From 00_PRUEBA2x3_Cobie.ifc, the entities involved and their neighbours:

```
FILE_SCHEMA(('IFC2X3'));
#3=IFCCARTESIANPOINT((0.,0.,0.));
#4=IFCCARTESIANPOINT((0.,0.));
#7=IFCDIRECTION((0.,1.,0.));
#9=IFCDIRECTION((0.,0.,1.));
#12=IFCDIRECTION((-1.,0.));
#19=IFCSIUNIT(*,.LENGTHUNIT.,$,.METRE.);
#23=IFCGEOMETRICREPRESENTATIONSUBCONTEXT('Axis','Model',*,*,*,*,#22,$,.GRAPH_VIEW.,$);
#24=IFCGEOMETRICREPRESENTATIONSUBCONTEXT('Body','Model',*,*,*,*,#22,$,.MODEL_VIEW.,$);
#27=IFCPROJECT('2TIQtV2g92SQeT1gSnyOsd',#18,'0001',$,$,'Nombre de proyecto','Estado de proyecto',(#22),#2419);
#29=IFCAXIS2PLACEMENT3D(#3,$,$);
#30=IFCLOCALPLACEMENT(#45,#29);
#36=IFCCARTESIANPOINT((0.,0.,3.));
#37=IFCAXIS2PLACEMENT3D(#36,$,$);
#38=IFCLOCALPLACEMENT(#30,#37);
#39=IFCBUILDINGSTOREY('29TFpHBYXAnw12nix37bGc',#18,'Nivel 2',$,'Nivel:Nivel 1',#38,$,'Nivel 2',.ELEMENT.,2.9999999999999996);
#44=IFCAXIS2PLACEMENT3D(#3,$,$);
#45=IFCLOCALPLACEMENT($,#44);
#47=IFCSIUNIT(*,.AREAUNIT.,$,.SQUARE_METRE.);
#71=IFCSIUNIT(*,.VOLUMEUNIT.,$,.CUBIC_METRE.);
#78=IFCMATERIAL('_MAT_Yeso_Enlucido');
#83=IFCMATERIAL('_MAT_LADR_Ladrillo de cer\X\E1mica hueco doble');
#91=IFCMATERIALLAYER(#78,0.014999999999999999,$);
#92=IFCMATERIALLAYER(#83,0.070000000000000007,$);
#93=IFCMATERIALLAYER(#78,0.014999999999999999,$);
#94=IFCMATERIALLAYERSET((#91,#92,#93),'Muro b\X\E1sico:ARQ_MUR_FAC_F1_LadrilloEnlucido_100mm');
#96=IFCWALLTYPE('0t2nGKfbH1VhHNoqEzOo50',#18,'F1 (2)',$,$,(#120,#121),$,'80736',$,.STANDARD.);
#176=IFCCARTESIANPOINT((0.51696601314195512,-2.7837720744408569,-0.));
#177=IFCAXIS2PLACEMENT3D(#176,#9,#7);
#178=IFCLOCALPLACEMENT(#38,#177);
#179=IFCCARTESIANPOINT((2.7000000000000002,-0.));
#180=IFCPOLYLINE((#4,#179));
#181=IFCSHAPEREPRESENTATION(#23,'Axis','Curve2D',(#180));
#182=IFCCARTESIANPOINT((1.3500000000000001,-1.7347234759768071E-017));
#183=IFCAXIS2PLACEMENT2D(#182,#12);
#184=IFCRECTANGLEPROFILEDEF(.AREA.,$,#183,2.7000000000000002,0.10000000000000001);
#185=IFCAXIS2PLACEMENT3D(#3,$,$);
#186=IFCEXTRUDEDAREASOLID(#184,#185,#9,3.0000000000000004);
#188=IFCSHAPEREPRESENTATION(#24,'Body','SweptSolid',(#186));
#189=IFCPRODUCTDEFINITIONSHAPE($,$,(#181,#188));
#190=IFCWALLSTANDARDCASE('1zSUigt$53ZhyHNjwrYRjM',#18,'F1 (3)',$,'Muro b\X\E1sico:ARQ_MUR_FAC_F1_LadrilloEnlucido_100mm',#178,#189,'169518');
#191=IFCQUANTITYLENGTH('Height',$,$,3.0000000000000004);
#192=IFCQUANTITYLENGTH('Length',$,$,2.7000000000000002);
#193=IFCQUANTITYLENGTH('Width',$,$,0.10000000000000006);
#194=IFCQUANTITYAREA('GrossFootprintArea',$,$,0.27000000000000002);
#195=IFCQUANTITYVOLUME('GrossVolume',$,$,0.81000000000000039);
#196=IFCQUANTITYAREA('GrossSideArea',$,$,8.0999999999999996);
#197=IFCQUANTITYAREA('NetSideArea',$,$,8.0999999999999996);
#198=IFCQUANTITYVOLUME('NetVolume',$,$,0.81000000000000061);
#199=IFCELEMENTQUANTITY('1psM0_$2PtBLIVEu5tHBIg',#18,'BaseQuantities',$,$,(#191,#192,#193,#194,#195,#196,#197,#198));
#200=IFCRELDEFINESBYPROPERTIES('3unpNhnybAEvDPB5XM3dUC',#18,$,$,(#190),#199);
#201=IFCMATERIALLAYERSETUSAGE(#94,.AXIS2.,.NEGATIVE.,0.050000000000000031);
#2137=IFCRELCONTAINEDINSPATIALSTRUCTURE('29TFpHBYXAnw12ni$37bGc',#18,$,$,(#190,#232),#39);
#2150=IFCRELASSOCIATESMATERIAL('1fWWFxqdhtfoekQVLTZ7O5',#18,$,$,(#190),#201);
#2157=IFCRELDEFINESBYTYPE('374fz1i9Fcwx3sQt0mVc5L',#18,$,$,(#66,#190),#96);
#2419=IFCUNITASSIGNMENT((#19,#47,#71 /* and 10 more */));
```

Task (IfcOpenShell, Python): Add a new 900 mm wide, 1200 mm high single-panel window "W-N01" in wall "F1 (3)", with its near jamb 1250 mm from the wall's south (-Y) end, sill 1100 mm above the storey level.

```python
import numpy as np
import ifcopenshell
import ifcopenshell.api.feature
import ifcopenshell.api.geometry
import ifcopenshell.api.pset
import ifcopenshell.api.root
import ifcopenshell.api.spatial
import ifcopenshell.api.type
import ifcopenshell.geom
import ifcopenshell.util.element
import ifcopenshell.util.placement
import ifcopenshell.util.representation
import ifcopenshell.util.shape
import ifcopenshell.util.unit

model = ifcopenshell.open("00_PRUEBA2x3_Cobie.ifc")
unit_scale = ifcopenshell.util.unit.calculate_unit_scale(model)
area_scale = ifcopenshell.util.unit.calculate_unit_scale(model, "AREAUNIT")
volume_scale = ifcopenshell.util.unit.calculate_unit_scale(model, "VOLUMEUNIT")
settings = ifcopenshell.geom.settings()


def volume(element):
    """Net volume in cubic metres, openings subtracted."""
    shape = ifcopenshell.geom.create_shape(settings, element)
    return ifcopenshell.util.shape.get_volume(shape.geometry)


wall = model.by_guid("1zSUigt$53ZhyHNjwrYRjM")
storey = ifcopenshell.util.element.get_container(wall, ifc_class="IfcBuildingStorey")
context = ifcopenshell.util.representation.get_context(model, "Model", "Body", "MODEL_VIEW")
before = volume(wall)

width, height, from_end, sill = 0.9, 1.2, 1.25, 1.1  # metres

# The wall runs along its own X axis, and the end named is its -X end.
wall_shape = ifcopenshell.geom.create_shape(settings, wall)
x, y, z = ifcopenshell.util.shape.get_vertices(wall_shape.geometry).T
start = x.min() + from_end
face, thickness = float(y.min()), float(y.max() - y.min())
wall_matrix = ifcopenshell.util.placement.get_local_placement(wall.ObjectPlacement)
level = ifcopenshell.util.placement.get_local_placement(storey.ObjectPlacement)[2, 3]


def in_wall(x, y):
    """Placement at x, y metres in the wall's axes, at sill height."""
    matrix = wall_matrix.copy()
    matrix[:, 3] = wall_matrix @ np.array([x / unit_scale, y / unit_scale, 0.0, 1.0])
    matrix[2, 3] = level + sill / unit_scale
    return matrix


# Opening: a box that overshoots both wall faces by 50 mm.
opening = ifcopenshell.api.root.create_entity(model, ifc_class="IfcOpeningElement")
box = ifcopenshell.api.geometry.add_wall_representation(
    model, context=context, length=width, height=height, thickness=thickness + 0.1
)
ifcopenshell.api.geometry.assign_representation(model, product=opening, representation=box)
ifcopenshell.api.geometry.edit_object_placement(model, product=opening, matrix=in_wall(start, face - 0.05), is_si=False)
ifcopenshell.api.feature.add_feature(model, feature=opening, element=wall)

window = ifcopenshell.api.root.create_entity(model, ifc_class="IfcWindow", name="W-N01")
window.OverallWidth, window.OverallHeight = width / unit_scale, height / unit_scale
body = ifcopenshell.api.geometry.add_window_representation(
    model,
    context=context,
    overall_width=window.OverallWidth,
    overall_height=window.OverallHeight,
    partition_type="SINGLE_PANEL",
)
ifcopenshell.api.geometry.assign_representation(model, product=window, representation=body)
ifcopenshell.api.spatial.assign_container(model, products=[window], relating_structure=storey)
fills = ifcopenshell.api.feature.add_filling(model, opening=opening, element=window)
fills.OwnerHistory = window.OwnerHistory  # required in IFC2X3

# IFC2X3 keeps the operation on the window style.
style = ifcopenshell.api.root.create_entity(model, ifc_class="IfcWindowStyle", name="W-N01")
style.OperationType, style.ConstructionType = "SINGLE_PANEL", "NOTDEFINED"
style.ParameterTakesPrecedence = style.Sizeable = False
ifcopenshell.api.type.assign_type(model, related_objects=[window], relating_type=style)

# Centre the window in the wall's thickness.
ifcopenshell.api.geometry.edit_object_placement(model, product=window, matrix=in_wall(start, face), is_si=False)
window_shape = ifcopenshell.geom.create_shape(settings, window)
depth = ifcopenshell.util.shape.get_vertices(window_shape.geometry)[:, 1]
offset = face + thickness / 2 - (depth.min() + depth.max()) / 2
ifcopenshell.api.geometry.edit_object_placement(model, product=window, matrix=in_wall(start, offset), is_si=False)

after = volume(wall)

# Update the wall's stored quantities.
qto = model.by_id(ifcopenshell.util.element.get_pset(wall, "BaseQuantities", should_inherit=False)["id"])
ifcopenshell.api.pset.edit_qto(model, qto=qto, properties={
    "NetSideArea": after / thickness / area_scale,
    "NetVolume": after / volume_scale,
})

print(f"wall volume {before:.3f} -> {after:.3f} m3")

model.write("00_PRUEBA2x3_Cobie_rev.ifc")
```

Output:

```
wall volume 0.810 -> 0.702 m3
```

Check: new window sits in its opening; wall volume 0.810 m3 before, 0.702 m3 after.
